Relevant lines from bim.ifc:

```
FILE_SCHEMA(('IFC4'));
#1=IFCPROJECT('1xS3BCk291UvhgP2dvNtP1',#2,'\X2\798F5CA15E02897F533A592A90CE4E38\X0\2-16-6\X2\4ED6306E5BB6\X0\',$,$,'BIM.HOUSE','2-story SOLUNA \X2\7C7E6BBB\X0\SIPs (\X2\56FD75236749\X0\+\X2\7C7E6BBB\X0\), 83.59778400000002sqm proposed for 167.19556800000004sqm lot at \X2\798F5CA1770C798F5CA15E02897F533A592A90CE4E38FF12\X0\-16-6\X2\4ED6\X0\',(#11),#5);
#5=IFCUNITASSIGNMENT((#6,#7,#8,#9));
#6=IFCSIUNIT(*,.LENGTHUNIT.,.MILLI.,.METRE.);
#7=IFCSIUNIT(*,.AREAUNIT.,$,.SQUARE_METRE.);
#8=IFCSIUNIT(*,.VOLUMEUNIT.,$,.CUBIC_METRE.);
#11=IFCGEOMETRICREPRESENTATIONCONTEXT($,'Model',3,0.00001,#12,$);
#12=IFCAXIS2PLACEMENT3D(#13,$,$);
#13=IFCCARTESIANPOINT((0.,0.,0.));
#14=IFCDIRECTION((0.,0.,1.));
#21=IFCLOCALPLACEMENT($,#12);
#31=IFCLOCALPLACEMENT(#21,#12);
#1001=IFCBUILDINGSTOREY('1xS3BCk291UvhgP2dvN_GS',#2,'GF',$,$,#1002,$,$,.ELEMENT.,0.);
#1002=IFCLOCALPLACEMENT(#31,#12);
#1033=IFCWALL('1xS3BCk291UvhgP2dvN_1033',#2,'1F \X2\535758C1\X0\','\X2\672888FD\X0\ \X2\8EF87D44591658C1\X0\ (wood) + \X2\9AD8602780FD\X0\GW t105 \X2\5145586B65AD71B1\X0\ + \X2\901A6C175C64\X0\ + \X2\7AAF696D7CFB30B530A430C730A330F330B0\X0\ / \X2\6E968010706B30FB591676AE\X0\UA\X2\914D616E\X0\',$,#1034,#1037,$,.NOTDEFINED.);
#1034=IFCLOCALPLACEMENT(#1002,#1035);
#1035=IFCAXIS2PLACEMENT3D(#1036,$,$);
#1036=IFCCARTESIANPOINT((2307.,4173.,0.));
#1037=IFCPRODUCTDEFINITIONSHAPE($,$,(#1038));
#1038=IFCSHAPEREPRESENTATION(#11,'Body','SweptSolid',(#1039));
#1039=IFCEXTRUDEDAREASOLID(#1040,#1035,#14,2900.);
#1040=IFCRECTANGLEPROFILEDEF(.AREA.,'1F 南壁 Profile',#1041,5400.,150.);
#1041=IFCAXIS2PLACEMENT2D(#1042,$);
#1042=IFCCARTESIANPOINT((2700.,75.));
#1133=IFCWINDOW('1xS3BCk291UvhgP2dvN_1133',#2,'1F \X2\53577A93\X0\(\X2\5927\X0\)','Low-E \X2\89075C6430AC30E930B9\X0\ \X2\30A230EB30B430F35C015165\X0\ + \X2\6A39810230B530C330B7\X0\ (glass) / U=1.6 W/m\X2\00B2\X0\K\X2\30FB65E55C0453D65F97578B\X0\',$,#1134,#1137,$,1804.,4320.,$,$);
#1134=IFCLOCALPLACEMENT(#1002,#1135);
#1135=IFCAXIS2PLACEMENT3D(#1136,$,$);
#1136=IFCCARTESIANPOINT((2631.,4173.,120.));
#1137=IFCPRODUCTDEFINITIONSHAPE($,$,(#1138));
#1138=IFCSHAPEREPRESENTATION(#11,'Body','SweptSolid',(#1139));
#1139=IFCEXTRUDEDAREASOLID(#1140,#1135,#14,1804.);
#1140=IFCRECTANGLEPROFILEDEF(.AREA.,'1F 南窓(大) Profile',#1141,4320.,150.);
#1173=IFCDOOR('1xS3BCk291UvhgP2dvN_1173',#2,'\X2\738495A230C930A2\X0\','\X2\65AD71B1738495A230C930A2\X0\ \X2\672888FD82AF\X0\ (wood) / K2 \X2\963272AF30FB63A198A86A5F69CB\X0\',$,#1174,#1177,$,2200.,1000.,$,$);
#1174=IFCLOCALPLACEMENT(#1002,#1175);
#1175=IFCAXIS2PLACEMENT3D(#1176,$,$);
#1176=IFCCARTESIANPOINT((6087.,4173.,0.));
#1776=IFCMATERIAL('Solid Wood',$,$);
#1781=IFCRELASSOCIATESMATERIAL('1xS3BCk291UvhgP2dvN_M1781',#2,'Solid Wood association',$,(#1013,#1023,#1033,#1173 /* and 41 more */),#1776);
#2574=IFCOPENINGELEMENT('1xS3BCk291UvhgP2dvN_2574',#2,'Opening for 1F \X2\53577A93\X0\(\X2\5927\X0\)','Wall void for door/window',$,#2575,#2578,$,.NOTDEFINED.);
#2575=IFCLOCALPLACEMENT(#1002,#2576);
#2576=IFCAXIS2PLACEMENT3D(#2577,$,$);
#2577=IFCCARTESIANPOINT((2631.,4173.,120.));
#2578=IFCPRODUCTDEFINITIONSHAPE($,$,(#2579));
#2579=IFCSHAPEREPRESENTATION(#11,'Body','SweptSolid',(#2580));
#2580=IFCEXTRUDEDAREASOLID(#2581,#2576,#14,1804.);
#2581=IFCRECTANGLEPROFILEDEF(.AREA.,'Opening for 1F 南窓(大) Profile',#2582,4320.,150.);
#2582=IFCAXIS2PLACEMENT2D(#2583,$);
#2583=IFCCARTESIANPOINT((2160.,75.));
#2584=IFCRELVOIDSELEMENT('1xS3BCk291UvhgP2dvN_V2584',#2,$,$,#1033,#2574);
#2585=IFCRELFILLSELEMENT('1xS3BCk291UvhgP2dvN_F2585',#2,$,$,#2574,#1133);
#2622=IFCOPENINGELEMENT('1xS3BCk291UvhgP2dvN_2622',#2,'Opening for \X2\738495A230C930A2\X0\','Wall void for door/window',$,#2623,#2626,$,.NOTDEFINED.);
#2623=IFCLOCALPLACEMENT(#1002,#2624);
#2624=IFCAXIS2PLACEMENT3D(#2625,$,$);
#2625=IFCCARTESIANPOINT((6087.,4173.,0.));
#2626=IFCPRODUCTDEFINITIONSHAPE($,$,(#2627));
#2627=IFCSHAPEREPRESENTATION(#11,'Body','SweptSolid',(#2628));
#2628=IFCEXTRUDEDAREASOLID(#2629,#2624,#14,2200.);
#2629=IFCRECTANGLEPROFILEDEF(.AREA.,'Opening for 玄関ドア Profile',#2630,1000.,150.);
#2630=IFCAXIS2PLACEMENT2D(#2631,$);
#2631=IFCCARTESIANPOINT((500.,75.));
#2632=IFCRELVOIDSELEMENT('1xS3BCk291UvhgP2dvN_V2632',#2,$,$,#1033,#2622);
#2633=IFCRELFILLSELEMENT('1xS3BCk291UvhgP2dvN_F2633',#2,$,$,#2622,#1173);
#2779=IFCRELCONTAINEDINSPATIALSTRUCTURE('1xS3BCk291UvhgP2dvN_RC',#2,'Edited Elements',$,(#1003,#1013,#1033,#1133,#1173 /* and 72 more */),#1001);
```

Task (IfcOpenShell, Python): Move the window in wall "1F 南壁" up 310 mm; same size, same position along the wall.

```python
import numpy as np
import ifcopenshell
import ifcopenshell.api.geometry
import ifcopenshell.util.placement
import ifcopenshell.util.unit

model = ifcopenshell.open("bim.ifc")
unit_scale = ifcopenshell.util.unit.calculate_unit_scale(model)

window = model.by_id(1133)
opening = window.FillsVoids[0].RelatingOpeningElement
dz = 310.0

shift = np.array([0.0, 0.0, dz])
# The window is not placed relative to its opening, so move both.
for product in (opening, window):
    matrix = ifcopenshell.util.placement.get_local_placement(product.ObjectPlacement)
    matrix[:3, 3] += shift
    ifcopenshell.api.geometry.edit_object_placement(model, product=product, matrix=matrix, is_si=False)

print(f"moved by {dz * unit_scale:+.3f} m")

model.write("bim_edited.ifc")
```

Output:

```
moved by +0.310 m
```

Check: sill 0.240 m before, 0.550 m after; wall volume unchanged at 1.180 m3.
